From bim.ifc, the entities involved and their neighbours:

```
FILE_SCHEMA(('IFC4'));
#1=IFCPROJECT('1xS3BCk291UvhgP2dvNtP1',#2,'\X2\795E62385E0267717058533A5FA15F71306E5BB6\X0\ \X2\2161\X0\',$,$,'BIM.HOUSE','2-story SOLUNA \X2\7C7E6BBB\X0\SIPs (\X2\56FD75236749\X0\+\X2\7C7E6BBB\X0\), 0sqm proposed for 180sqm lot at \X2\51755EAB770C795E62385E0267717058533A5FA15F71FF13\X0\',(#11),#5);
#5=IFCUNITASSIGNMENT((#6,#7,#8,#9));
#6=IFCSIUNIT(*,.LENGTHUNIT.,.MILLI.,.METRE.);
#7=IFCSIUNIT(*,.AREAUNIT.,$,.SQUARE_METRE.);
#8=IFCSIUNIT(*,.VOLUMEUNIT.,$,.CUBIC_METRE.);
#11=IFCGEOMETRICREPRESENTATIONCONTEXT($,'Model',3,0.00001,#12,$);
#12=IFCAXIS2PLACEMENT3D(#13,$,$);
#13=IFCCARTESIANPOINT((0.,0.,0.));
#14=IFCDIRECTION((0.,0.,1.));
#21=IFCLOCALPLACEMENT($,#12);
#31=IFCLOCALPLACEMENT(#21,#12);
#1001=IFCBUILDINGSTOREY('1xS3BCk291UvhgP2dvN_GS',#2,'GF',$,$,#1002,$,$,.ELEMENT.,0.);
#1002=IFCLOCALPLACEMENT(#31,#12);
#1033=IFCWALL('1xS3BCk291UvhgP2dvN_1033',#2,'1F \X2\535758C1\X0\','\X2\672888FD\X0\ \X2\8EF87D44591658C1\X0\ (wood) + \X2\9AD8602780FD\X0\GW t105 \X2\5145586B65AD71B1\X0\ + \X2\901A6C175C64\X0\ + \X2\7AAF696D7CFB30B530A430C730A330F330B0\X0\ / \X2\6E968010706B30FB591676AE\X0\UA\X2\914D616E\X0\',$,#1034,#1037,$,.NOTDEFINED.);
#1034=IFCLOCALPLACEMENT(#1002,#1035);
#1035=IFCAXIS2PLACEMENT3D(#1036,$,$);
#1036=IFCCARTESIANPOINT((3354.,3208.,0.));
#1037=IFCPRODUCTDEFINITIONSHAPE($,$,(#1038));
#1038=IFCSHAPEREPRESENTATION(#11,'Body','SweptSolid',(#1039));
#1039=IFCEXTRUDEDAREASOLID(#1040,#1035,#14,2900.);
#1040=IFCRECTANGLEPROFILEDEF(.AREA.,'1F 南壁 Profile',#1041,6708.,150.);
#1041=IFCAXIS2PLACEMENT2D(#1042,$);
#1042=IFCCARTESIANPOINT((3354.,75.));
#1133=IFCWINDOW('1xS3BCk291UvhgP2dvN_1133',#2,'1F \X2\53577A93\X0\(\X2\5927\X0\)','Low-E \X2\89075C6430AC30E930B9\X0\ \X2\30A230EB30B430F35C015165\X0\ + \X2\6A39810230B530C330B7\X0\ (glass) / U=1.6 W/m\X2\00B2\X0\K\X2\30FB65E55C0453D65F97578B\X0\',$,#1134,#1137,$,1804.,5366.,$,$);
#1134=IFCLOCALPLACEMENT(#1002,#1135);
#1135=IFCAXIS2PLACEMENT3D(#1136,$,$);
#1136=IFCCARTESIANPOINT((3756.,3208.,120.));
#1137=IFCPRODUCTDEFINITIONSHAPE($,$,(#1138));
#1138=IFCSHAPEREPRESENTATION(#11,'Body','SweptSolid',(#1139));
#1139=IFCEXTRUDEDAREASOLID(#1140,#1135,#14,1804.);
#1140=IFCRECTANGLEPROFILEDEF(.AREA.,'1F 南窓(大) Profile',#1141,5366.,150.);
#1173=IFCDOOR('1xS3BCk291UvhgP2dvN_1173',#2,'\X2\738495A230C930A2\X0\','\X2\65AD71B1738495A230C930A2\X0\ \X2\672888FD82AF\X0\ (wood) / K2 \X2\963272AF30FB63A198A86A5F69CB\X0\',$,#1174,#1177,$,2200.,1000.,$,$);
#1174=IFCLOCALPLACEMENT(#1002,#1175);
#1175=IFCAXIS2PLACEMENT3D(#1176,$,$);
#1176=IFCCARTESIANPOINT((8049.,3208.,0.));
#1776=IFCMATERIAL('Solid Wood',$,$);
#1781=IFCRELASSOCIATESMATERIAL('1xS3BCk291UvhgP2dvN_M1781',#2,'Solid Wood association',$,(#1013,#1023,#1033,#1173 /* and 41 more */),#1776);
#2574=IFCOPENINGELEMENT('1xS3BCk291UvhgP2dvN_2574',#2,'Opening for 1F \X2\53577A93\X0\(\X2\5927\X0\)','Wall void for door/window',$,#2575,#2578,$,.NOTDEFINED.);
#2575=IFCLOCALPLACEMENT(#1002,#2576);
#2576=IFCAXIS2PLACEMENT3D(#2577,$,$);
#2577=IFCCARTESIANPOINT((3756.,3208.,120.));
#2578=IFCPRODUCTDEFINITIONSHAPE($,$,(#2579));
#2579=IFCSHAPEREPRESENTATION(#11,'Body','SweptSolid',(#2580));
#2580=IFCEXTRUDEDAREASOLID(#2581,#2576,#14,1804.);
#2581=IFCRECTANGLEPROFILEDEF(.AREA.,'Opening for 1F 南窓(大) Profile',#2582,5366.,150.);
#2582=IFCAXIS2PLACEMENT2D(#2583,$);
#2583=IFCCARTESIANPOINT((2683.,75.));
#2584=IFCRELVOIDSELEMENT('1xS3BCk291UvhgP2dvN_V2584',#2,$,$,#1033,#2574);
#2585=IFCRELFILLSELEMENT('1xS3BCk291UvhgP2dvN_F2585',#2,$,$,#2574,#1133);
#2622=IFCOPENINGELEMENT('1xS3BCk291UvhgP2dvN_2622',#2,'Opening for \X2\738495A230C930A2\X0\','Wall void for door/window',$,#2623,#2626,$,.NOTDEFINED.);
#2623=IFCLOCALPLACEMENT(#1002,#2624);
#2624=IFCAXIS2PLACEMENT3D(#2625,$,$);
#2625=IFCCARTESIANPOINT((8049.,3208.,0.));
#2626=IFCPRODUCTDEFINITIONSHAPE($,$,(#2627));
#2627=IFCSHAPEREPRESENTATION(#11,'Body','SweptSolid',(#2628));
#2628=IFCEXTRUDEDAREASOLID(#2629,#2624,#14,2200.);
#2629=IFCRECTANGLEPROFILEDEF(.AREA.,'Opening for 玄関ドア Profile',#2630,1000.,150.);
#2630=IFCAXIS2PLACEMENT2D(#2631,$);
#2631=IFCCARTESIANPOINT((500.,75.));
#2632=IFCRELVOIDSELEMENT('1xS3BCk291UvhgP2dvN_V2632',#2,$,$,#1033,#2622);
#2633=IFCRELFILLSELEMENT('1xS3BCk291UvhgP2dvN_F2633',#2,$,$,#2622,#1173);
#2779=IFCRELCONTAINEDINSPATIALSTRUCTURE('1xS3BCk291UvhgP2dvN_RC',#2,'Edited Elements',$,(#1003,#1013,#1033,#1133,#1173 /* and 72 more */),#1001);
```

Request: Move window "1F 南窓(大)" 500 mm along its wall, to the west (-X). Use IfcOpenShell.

```python
import ifcopenshell
import ifcopenshell.api.geometry
import ifcopenshell.util.placement

model = ifcopenshell.open("bim.ifc")

window = model.by_guid("1xS3BCk291UvhgP2dvN_1133")
opening = window.FillsVoids[0].RelatingOpeningElement
wall = opening.VoidsElements[0].RelatingBuildingElement

wall_matrix = ifcopenshell.util.placement.get_local_placement(wall.ObjectPlacement)
shift = wall_matrix[:3, 0] * -500.0
before = ifcopenshell.util.placement.get_local_placement(window.ObjectPlacement)[:3, 3].copy()

# The window is not placed relative to its opening, so move both.
for product in (opening, window):
    matrix = ifcopenshell.util.placement.get_local_placement(product.ObjectPlacement)
    matrix[:3, 3] += shift
    ifcopenshell.api.geometry.edit_object_placement(model, product=product, matrix=matrix, is_si=False)

after = ifcopenshell.util.placement.get_local_placement(window.ObjectPlacement)[:3, 3]
print("window moved by", (after - before).round(3) + 0.0)

model.write("bim_edited.ifc")
```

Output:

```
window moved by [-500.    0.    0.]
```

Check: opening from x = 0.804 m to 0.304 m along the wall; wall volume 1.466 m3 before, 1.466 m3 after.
